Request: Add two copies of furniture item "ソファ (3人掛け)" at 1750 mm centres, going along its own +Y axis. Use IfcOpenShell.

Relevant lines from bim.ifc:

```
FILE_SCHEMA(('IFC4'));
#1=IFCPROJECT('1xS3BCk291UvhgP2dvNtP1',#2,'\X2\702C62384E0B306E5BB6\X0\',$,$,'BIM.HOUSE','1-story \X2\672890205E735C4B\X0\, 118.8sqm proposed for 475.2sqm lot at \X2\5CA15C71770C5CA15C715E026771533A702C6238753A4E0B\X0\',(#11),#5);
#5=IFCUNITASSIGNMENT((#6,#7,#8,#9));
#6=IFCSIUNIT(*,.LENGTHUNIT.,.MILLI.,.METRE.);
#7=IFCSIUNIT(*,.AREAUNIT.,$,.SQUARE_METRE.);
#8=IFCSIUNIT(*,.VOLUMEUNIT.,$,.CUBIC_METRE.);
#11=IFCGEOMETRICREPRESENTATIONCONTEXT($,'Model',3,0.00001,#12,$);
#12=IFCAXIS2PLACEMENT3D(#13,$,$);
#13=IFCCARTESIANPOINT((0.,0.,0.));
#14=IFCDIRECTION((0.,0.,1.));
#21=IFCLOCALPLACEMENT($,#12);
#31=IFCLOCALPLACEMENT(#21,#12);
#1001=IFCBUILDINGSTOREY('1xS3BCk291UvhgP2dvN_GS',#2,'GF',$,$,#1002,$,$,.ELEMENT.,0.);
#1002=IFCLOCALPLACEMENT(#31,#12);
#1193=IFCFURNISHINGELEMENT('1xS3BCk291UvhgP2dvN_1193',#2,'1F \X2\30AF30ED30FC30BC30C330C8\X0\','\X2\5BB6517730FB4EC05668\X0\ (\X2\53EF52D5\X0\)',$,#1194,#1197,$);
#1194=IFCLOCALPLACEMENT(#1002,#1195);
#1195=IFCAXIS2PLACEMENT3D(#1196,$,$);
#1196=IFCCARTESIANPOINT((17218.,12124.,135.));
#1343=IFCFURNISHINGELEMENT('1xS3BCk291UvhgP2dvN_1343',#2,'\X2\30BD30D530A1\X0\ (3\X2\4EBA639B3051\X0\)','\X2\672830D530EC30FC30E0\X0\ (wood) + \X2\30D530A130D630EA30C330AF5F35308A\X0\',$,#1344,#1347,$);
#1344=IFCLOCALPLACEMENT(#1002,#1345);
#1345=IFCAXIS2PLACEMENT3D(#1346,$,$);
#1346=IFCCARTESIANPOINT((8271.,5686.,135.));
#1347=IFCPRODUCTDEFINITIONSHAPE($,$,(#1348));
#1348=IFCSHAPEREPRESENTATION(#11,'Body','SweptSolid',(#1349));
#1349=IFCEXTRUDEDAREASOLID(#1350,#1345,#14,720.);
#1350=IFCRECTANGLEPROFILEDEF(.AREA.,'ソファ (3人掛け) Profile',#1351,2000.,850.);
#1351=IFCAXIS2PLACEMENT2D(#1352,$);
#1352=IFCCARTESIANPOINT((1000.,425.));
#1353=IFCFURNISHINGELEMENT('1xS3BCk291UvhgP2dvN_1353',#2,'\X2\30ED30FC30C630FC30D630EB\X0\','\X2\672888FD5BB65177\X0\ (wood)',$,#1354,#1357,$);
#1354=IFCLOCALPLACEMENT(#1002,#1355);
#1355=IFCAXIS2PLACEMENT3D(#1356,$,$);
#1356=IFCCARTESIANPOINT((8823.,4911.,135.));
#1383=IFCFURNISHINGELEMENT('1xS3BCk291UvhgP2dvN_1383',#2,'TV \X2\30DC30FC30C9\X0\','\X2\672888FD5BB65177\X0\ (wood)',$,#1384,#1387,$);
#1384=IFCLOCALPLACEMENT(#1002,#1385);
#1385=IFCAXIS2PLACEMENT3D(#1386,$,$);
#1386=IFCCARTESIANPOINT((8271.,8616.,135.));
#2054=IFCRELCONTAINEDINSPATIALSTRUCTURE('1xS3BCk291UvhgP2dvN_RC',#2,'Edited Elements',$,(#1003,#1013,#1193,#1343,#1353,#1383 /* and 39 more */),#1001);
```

```python
import ifcopenshell
import ifcopenshell.api.geometry
import ifcopenshell.api.root
import ifcopenshell.util.element
import ifcopenshell.util.placement
import ifcopenshell.util.unit

model = ifcopenshell.open("bim.ifc")
unit_scale = ifcopenshell.util.unit.calculate_unit_scale(model)


def reuse_history(source, copy):
    """copy_class also copies each property set's owner history, people and application; keep the originals."""
    for rel in copy.IsDefinedBy:
        if rel.is_a("IfcRelDefinesByProperties") and (history := rel.RelatingPropertyDefinition.OwnerHistory):
            rel.RelatingPropertyDefinition.OwnerHistory = source.OwnerHistory
            ifcopenshell.util.element.remove_deep2(model, history)


source = model.by_id(1343)
base = ifcopenshell.util.placement.get_local_placement(source.ObjectPlacement)
step = base[:3, 1] * 1.75 / unit_scale

for i in range(1, 3):
    copy = ifcopenshell.api.root.copy_class(model, product=source)
    copy.Representation = ifcopenshell.util.element.copy_deep(
        model, source.Representation, exclude=["IfcGeometricRepresentationContext", "IfcRepresentationMap"]
    )
    reuse_history(source, copy)
    matrix = base.copy()
    matrix[:3, 3] += i * step
    print("added at", matrix[:3, 3].round(3) + 0.0)
    ifcopenshell.api.geometry.edit_object_placement(model, product=copy, matrix=matrix, is_si=False)

model.write("bim_rev.ifc")
```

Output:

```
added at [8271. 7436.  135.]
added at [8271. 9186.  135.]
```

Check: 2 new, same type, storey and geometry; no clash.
